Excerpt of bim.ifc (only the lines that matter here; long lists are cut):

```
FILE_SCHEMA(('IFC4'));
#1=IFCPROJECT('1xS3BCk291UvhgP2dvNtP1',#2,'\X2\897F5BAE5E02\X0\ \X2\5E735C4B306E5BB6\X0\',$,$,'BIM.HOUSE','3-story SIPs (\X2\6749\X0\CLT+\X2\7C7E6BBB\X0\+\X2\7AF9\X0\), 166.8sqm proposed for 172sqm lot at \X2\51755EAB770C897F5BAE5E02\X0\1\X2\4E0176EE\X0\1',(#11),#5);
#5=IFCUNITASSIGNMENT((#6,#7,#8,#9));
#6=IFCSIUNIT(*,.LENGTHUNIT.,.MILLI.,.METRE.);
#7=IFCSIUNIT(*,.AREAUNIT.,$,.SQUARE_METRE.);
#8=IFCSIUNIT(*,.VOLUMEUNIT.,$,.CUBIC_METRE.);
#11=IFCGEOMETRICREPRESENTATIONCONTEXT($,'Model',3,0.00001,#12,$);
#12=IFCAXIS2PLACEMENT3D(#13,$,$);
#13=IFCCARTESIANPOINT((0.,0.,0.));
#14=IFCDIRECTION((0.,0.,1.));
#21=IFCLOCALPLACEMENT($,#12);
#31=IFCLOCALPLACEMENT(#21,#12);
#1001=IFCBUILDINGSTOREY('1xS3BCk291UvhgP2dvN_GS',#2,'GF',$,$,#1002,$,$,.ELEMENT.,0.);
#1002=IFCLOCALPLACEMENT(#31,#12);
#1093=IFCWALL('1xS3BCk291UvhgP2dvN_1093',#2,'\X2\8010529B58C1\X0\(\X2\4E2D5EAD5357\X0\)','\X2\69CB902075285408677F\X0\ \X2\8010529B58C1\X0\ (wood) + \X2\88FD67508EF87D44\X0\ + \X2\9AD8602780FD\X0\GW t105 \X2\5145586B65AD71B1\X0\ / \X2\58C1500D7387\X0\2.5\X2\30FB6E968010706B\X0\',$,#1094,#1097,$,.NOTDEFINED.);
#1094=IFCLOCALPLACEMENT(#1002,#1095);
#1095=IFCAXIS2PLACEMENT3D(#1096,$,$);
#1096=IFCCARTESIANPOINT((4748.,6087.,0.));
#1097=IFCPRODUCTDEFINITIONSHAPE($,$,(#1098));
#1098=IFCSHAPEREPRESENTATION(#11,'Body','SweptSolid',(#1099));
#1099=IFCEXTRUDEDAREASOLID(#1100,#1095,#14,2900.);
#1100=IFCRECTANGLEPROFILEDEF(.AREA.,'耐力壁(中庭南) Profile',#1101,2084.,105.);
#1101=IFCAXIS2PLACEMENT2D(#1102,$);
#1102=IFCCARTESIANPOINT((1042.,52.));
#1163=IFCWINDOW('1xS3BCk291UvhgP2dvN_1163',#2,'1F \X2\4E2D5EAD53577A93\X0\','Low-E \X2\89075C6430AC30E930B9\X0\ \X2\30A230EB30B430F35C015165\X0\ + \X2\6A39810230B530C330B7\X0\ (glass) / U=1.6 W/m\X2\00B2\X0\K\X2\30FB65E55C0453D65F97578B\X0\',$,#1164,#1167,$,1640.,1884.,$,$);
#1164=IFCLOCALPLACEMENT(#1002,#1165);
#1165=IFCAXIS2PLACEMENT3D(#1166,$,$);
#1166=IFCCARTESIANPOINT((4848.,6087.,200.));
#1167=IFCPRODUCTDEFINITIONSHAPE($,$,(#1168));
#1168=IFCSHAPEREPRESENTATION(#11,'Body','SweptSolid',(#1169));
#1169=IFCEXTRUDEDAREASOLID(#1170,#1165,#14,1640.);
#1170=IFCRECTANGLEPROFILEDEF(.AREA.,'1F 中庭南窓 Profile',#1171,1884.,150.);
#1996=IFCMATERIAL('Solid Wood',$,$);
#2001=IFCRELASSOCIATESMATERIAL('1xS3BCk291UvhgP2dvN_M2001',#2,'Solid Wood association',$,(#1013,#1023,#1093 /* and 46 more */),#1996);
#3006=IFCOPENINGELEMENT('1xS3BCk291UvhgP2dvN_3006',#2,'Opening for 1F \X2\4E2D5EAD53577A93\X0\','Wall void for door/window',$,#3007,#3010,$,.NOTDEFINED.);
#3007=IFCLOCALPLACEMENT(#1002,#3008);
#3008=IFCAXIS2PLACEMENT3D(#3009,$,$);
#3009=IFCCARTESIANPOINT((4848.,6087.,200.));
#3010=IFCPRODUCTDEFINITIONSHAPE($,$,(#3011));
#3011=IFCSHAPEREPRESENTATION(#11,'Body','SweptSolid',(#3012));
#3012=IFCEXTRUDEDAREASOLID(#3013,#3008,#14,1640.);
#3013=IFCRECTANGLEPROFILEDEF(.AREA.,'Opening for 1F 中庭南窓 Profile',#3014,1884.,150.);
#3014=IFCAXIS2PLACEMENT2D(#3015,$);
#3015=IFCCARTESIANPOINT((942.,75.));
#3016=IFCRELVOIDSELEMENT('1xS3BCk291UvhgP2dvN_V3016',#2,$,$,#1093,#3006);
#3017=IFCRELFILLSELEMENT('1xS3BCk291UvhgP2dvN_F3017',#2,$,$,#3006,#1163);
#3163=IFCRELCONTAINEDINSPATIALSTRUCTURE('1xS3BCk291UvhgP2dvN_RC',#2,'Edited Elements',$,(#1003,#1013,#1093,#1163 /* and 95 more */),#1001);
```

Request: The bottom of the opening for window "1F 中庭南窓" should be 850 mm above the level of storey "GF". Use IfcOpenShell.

```python
import numpy as np
import ifcopenshell
import ifcopenshell.api.geometry
import ifcopenshell.geom
import ifcopenshell.util.element
import ifcopenshell.util.placement
import ifcopenshell.util.shape
import ifcopenshell.util.unit

model = ifcopenshell.open("bim.ifc")
unit_scale = ifcopenshell.util.unit.calculate_unit_scale(model)

window = model.by_id(1163)
opening = window.FillsVoids[0].RelatingOpeningElement
storey = ifcopenshell.util.element.get_container(window, ifc_class="IfcBuildingStorey")
level = ifcopenshell.util.placement.get_local_placement(storey.ObjectPlacement)[2, 3]

# The opening's origin need not be at the sill, so measure its lowest point.
shape = ifcopenshell.geom.create_shape(ifcopenshell.geom.settings(), opening)
bottom = ifcopenshell.util.shape.get_shape_bottom_elevation(shape, shape.geometry) / unit_scale
dz = level + 0.85 / unit_scale - bottom

shift = np.array([0.0, 0.0, dz])
# The window is not placed relative to its opening, so move both.
for product in (opening, window):
    matrix = ifcopenshell.util.placement.get_local_placement(product.ObjectPlacement)
    matrix[:3, 3] += shift
    ifcopenshell.api.geometry.edit_object_placement(model, product=product, matrix=matrix, is_si=False)

print(f"moved by {dz * unit_scale:+.3f} m")

model.write("bim_v2.ifc")
```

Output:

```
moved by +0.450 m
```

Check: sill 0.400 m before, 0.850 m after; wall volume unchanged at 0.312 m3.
